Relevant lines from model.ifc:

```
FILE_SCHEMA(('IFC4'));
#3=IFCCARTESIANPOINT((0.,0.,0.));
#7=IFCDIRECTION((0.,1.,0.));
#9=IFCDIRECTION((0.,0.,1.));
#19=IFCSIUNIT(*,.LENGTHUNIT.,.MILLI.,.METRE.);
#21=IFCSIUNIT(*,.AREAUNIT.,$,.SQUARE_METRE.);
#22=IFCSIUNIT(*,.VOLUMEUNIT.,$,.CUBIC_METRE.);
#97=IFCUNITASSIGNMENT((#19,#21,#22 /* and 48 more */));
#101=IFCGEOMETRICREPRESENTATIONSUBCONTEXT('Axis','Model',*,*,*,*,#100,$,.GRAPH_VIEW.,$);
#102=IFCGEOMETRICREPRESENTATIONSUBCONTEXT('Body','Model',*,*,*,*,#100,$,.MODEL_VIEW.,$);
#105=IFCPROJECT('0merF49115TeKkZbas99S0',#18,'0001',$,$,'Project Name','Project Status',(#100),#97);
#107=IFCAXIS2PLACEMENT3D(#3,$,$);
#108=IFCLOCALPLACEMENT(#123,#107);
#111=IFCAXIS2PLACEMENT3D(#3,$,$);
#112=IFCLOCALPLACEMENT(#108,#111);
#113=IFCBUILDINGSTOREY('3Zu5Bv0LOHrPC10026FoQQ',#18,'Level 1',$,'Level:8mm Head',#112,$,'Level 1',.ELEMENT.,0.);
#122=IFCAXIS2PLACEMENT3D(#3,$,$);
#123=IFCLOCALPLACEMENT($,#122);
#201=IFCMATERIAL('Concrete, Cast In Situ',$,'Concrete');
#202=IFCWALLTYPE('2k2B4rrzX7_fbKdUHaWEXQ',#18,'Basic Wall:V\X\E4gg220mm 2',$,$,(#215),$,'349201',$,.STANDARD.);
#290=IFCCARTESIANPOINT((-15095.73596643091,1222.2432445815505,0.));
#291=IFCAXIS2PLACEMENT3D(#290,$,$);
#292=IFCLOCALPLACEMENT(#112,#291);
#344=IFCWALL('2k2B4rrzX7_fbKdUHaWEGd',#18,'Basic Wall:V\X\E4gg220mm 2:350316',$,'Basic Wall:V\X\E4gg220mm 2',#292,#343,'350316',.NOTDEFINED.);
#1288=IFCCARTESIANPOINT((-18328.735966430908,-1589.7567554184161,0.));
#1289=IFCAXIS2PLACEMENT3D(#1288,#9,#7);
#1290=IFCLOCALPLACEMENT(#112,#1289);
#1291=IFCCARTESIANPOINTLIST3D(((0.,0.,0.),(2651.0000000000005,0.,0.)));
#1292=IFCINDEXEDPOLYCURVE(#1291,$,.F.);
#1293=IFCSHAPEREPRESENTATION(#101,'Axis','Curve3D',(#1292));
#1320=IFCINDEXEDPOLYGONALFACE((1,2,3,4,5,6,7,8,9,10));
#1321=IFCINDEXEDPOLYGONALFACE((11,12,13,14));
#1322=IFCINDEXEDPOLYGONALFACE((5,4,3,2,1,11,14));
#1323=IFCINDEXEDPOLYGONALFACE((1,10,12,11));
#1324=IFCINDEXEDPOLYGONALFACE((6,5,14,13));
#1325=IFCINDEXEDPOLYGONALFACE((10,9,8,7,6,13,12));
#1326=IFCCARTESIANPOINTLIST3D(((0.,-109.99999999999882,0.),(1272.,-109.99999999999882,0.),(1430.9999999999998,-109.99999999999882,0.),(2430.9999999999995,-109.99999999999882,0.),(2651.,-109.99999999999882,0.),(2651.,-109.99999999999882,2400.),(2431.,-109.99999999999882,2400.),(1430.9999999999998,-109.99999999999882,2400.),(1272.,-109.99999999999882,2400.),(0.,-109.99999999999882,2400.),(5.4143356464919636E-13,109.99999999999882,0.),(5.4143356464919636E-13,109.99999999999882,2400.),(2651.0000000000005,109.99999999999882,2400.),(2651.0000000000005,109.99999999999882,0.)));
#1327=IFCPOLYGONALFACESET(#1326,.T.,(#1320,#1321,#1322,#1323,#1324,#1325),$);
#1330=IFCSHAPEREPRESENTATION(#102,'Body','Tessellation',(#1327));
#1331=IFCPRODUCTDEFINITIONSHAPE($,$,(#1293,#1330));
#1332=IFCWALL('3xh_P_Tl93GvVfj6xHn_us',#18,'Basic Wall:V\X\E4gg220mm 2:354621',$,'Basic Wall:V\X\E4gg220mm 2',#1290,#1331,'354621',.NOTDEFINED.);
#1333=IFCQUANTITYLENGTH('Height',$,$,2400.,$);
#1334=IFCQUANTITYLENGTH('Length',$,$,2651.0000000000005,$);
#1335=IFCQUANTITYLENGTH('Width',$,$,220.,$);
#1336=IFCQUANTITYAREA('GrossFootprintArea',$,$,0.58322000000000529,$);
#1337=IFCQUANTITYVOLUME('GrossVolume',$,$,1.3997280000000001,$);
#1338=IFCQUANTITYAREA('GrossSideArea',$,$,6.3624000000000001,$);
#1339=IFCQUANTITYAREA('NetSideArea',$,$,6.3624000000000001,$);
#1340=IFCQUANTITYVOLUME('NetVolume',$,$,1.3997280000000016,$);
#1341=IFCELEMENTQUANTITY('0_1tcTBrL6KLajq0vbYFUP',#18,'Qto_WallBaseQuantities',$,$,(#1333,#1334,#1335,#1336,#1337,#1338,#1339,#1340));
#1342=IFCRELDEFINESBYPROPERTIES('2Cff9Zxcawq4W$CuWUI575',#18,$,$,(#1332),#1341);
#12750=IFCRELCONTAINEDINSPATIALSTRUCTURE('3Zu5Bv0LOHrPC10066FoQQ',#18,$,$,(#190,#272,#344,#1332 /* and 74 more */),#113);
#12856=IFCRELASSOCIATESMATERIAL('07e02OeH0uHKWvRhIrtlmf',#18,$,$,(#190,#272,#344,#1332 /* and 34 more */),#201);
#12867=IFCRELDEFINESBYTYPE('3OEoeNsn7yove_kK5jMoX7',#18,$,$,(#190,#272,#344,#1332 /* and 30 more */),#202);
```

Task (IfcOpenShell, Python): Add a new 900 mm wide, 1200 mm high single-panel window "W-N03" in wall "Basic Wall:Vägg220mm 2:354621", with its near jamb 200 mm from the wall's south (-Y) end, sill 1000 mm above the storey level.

```python
import numpy as np
import ifcopenshell
import ifcopenshell.api.feature
import ifcopenshell.api.geometry
import ifcopenshell.api.pset
import ifcopenshell.api.root
import ifcopenshell.api.spatial
import ifcopenshell.geom
import ifcopenshell.util.element
import ifcopenshell.util.placement
import ifcopenshell.util.representation
import ifcopenshell.util.shape
import ifcopenshell.util.unit

model = ifcopenshell.open("model.ifc")
unit_scale = ifcopenshell.util.unit.calculate_unit_scale(model)
area_scale = ifcopenshell.util.unit.calculate_unit_scale(model, "AREAUNIT")
volume_scale = ifcopenshell.util.unit.calculate_unit_scale(model, "VOLUMEUNIT")
settings = ifcopenshell.geom.settings()


def volume(element):
    """Net volume in cubic metres, openings subtracted."""
    shape = ifcopenshell.geom.create_shape(settings, element)
    return ifcopenshell.util.shape.get_volume(shape.geometry)


wall = model.by_guid("3xh_P_Tl93GvVfj6xHn_us")
storey = ifcopenshell.util.element.get_container(wall, ifc_class="IfcBuildingStorey")
context = ifcopenshell.util.representation.get_context(model, "Model", "Body", "MODEL_VIEW")
before = volume(wall)

width, height, from_end, sill = 0.9, 1.2, 0.2, 1  # metres

# The wall runs along its own X axis, and the end named is its -X end.
wall_shape = ifcopenshell.geom.create_shape(settings, wall)
x, y, z = ifcopenshell.util.shape.get_vertices(wall_shape.geometry).T
start = x.min() + from_end
face, thickness = float(y.min()), float(y.max() - y.min())
wall_matrix = ifcopenshell.util.placement.get_local_placement(wall.ObjectPlacement)
level = ifcopenshell.util.placement.get_local_placement(storey.ObjectPlacement)[2, 3]


def in_wall(x, y):
    """Placement at x, y metres in the wall's axes, at sill height."""
    matrix = wall_matrix.copy()
    matrix[:, 3] = wall_matrix @ np.array([x / unit_scale, y / unit_scale, 0.0, 1.0])
    matrix[2, 3] = level + sill / unit_scale
    return matrix


# Opening: a box that overshoots both wall faces by 50 mm.
opening = ifcopenshell.api.root.create_entity(model, ifc_class="IfcOpeningElement", predefined_type="OPENING")
box = ifcopenshell.api.geometry.add_wall_representation(
    model, context=context, length=width, height=height, thickness=thickness + 0.1
)
ifcopenshell.api.geometry.assign_representation(model, product=opening, representation=box)
ifcopenshell.api.geometry.edit_object_placement(model, product=opening, matrix=in_wall(start, face - 0.05), is_si=False)
ifcopenshell.api.feature.add_feature(model, feature=opening, element=wall)

window = ifcopenshell.api.root.create_entity(model, ifc_class="IfcWindow", name="W-N03", predefined_type="WINDOW")
window.OverallWidth, window.OverallHeight = width / unit_scale, height / unit_scale
window.PartitioningType = "SINGLE_PANEL"
body = ifcopenshell.api.geometry.add_window_representation(
    model,
    context=context,
    overall_width=window.OverallWidth,
    overall_height=window.OverallHeight,
    partition_type="SINGLE_PANEL",
)
ifcopenshell.api.geometry.assign_representation(model, product=window, representation=body)
ifcopenshell.api.spatial.assign_container(model, products=[window], relating_structure=storey)
ifcopenshell.api.feature.add_filling(model, opening=opening, element=window)

# Centre the window in the wall's thickness.
ifcopenshell.api.geometry.edit_object_placement(model, product=window, matrix=in_wall(start, face), is_si=False)
window_shape = ifcopenshell.geom.create_shape(settings, window)
depth = ifcopenshell.util.shape.get_vertices(window_shape.geometry)[:, 1]
offset = face + thickness / 2 - (depth.min() + depth.max()) / 2
ifcopenshell.api.geometry.edit_object_placement(model, product=window, matrix=in_wall(start, offset), is_si=False)

after = volume(wall)

# Update the wall's stored quantities.
qto = model.by_id(ifcopenshell.util.element.get_pset(wall, "Qto_WallBaseQuantities", should_inherit=False)["id"])
ifcopenshell.api.pset.edit_qto(model, qto=qto, properties={
    "NetSideArea": after / thickness / area_scale,
    "NetVolume": after / volume_scale,
})

print(f"wall volume {before:.3f} -> {after:.3f} m3")

model.write("model_updated.ifc")
```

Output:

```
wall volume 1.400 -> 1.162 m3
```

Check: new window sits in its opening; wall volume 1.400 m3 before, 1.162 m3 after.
